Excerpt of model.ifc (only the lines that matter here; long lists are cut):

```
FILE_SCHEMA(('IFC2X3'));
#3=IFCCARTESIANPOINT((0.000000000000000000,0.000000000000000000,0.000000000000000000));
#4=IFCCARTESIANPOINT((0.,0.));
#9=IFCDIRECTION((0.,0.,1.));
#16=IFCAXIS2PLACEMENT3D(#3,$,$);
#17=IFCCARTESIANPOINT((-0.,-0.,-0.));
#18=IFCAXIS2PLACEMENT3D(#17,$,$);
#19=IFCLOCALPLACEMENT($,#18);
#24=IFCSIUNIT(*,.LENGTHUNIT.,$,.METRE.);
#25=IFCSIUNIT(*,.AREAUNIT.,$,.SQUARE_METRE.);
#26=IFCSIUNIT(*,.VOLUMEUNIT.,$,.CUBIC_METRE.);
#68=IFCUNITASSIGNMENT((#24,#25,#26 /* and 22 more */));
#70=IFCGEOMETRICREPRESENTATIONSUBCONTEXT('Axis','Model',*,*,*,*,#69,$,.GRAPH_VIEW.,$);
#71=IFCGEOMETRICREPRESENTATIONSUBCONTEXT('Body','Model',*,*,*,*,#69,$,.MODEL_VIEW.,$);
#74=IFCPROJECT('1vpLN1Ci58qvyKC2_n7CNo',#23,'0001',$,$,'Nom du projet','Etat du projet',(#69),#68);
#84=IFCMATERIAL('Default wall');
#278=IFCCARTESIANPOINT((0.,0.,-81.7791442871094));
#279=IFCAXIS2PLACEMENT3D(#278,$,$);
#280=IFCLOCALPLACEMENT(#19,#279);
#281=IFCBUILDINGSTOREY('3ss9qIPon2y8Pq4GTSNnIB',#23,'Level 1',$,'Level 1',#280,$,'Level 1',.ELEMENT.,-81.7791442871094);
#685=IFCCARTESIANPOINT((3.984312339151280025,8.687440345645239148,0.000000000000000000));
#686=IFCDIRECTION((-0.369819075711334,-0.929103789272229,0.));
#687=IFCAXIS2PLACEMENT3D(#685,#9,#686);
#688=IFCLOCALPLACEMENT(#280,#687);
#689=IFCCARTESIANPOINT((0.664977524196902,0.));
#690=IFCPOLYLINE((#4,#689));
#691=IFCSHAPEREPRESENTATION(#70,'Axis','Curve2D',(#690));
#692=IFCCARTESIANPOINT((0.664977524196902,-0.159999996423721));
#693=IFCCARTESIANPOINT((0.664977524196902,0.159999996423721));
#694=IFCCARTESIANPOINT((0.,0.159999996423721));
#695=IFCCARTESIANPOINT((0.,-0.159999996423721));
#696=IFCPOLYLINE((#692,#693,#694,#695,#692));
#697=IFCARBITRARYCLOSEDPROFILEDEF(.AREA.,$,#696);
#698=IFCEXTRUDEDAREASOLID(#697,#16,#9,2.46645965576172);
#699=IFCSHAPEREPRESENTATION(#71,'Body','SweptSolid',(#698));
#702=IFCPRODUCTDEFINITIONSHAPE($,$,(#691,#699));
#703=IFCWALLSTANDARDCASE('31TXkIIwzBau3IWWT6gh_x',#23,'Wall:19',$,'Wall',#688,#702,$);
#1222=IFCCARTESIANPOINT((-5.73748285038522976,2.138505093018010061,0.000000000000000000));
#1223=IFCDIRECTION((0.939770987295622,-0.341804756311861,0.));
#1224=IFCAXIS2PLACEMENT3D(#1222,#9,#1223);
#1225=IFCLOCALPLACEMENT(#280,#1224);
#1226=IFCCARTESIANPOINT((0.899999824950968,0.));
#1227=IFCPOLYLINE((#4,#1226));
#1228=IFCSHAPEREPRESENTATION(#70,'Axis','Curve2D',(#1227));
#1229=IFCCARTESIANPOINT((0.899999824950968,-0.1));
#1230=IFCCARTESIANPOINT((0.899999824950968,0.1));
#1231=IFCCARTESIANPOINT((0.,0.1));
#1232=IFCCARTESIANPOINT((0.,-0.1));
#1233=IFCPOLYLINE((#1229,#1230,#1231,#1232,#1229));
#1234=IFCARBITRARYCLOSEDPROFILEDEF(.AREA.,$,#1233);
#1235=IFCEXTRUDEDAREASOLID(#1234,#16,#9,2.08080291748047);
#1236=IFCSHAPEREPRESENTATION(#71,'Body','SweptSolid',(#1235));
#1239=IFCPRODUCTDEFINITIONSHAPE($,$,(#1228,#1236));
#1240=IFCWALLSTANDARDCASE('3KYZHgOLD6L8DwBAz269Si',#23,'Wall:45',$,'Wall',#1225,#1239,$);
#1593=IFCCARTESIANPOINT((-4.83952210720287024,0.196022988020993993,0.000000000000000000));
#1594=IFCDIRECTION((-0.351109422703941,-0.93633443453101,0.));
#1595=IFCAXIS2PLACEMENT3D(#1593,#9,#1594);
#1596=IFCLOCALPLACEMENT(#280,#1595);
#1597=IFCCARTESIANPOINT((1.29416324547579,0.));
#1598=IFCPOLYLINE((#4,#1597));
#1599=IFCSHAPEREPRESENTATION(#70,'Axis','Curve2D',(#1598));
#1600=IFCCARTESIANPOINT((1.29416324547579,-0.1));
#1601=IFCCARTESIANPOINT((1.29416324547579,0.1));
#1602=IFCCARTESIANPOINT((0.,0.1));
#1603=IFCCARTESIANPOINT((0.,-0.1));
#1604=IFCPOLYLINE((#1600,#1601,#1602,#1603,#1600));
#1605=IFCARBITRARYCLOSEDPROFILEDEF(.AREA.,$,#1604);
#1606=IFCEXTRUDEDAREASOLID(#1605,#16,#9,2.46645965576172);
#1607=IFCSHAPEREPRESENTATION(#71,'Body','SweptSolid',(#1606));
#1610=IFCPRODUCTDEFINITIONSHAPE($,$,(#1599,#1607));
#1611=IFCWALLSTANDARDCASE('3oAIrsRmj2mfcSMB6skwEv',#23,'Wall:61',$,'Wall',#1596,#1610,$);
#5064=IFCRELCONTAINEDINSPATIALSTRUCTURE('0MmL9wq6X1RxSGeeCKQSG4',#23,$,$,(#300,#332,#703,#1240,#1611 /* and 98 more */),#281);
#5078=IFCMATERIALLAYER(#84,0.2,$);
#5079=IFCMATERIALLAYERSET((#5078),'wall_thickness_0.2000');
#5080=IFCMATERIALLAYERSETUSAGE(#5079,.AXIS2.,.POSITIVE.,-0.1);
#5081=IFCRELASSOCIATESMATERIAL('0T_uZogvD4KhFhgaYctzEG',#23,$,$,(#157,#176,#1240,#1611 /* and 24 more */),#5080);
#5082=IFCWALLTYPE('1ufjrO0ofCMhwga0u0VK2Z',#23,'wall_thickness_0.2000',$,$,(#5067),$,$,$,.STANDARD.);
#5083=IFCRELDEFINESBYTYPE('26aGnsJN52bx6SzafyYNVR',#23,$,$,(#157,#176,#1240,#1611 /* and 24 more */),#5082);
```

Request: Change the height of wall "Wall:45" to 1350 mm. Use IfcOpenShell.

```python
import ifcopenshell
import ifcopenshell.geom
import ifcopenshell.util.representation
import ifcopenshell.util.shape
import ifcopenshell.util.unit

model = ifcopenshell.open("model.ifc")
unit_scale = ifcopenshell.util.unit.calculate_unit_scale(model)
settings = ifcopenshell.geom.settings()


def volume(element):
    """Net volume in cubic metres, openings subtracted."""
    shape = ifcopenshell.geom.create_shape(settings, element)
    return ifcopenshell.util.shape.get_volume(shape.geometry)


wall = model.by_guid("3KYZHgOLD6L8DwBAz269Si")
before = volume(wall)

body = ifcopenshell.util.representation.get_representation(wall, "Model", "Body")
solid = body.Items[0]
old_height = solid.Depth
solid.Depth = 1.35 / unit_scale
after = volume(wall)

print(f"height {old_height:g} -> {solid.Depth:g}, volume {before:.3f} -> {after:.3f} m3")

model.write("model-out.ifc")
```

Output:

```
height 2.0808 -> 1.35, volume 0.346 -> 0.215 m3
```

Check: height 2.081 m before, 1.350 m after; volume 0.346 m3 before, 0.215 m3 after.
